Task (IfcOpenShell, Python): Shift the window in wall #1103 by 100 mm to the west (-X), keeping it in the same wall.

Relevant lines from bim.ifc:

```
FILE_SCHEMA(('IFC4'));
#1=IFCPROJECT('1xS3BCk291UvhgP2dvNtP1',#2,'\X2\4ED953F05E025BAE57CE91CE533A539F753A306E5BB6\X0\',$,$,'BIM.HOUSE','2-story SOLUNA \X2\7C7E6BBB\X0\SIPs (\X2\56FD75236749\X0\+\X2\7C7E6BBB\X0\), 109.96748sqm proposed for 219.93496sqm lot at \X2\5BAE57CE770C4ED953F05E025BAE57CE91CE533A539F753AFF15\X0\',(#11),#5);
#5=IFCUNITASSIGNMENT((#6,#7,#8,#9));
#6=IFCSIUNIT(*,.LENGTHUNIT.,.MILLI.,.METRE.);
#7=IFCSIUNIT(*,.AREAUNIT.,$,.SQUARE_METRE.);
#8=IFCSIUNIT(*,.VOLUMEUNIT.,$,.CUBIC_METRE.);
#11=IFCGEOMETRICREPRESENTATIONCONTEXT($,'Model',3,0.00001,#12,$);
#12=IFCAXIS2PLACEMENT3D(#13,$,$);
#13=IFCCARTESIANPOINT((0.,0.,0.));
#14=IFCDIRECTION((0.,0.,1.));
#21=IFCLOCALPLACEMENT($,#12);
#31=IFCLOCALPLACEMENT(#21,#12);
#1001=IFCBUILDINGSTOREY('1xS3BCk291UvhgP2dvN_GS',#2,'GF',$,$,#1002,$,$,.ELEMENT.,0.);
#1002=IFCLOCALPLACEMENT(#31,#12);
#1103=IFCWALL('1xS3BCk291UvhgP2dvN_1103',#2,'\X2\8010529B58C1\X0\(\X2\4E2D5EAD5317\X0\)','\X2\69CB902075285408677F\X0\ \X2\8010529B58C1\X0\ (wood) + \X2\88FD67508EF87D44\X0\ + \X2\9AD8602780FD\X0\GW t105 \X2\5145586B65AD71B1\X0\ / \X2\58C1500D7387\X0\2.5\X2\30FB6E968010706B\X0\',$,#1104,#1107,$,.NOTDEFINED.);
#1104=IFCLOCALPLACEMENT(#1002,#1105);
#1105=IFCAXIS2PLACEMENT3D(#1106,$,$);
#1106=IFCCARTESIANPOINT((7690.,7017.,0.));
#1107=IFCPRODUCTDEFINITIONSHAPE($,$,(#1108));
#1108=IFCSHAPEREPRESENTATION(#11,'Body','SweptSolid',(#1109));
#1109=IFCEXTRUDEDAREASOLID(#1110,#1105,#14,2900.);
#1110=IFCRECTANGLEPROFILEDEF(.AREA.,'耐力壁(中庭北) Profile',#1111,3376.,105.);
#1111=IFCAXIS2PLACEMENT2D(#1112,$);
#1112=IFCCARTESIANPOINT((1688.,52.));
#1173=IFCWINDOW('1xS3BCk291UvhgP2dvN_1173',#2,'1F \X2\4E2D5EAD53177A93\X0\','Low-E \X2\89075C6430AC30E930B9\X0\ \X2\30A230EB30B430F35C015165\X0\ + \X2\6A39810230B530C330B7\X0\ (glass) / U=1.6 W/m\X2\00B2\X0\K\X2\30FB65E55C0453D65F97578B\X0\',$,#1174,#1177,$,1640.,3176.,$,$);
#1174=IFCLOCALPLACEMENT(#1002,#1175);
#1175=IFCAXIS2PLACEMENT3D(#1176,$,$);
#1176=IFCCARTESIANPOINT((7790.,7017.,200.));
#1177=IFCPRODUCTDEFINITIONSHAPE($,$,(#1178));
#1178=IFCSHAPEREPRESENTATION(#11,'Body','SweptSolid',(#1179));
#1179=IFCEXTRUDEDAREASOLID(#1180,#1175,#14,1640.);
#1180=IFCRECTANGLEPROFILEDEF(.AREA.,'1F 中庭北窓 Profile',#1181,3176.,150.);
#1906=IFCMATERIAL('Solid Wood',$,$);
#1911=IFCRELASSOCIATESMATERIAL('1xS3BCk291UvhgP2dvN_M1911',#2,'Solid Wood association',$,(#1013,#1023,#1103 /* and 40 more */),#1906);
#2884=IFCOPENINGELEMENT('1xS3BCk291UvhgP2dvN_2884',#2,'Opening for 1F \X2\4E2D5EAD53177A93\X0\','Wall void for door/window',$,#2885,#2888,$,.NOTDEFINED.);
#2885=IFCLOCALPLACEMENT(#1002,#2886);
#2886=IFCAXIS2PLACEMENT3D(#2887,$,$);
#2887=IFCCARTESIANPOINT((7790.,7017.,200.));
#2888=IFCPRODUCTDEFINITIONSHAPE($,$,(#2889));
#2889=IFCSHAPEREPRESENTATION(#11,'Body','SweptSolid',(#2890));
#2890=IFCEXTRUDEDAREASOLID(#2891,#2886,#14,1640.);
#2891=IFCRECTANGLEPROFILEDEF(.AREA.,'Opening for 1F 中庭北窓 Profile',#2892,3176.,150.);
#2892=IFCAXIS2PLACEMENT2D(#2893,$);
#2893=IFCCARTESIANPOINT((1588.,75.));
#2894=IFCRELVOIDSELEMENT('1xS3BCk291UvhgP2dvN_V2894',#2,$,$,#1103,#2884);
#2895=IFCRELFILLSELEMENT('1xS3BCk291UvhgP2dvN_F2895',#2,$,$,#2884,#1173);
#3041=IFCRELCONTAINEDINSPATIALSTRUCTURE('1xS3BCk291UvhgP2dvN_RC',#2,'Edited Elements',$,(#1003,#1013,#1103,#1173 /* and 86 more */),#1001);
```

```python
import ifcopenshell
import ifcopenshell.api.geometry
import ifcopenshell.util.placement
import ifcopenshell.util.unit

model = ifcopenshell.open("bim.ifc")
unit_scale = ifcopenshell.util.unit.calculate_unit_scale(model)

window = model.by_id(1173)
opening = window.FillsVoids[0].RelatingOpeningElement
wall = opening.VoidsElements[0].RelatingBuildingElement

wall_matrix = ifcopenshell.util.placement.get_local_placement(wall.ObjectPlacement)
shift = wall_matrix[:3, 0] * -0.1 / unit_scale
before = ifcopenshell.util.placement.get_local_placement(window.ObjectPlacement)[:3, 3].copy()

# The window is not placed relative to its opening, so move both.
for product in (opening, window):
    matrix = ifcopenshell.util.placement.get_local_placement(product.ObjectPlacement)
    matrix[:3, 3] += shift
    ifcopenshell.api.geometry.edit_object_placement(model, product=product, matrix=matrix, is_si=False)

after = ifcopenshell.util.placement.get_local_placement(window.ObjectPlacement)[:3, 3]
print("window moved by", (after - before).round(3) + 0.0)

model.write("bim_rev.ifc")
```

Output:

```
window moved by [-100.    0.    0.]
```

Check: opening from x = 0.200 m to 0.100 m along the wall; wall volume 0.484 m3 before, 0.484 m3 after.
